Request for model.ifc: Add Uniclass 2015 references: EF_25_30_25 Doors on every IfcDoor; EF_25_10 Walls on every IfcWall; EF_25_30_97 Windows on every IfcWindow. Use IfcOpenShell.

First a look at what the model holds.

```python
import ifcopenshell

model = ifcopenshell.open("model.ifc")
print(model.schema)
print("classifications:", [c.Name for c in model.by_type("IfcClassification")])
for ifc_class in ("IfcDoor", "IfcRoof", "IfcStair", "IfcWall", "IfcWindow"):
    print(ifc_class, len(model.by_type(ifc_class)))
```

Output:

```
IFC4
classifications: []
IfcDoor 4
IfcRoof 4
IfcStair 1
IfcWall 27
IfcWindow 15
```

```python
import ifcopenshell
import ifcopenshell.api.classification

model = ifcopenshell.open("model.ifc")

system = ifcopenshell.api.classification.add_classification(model, classification="Uniclass 2015")

codes = {
    "IfcDoor": ("EF_25_30_25", "Doors"),
    "IfcWall": ("EF_25_10", "Walls"),
    "IfcWindow": ("EF_25_30_97", "Windows"),
}
for ifc_class, (code, name) in codes.items():
    products = model.by_type(ifc_class)
    ifcopenshell.api.classification.add_reference(
        model, products=products, classification=system, identification=code, name=name
    )
    print(code, len(products))

model.write("model_edited.ifc")
```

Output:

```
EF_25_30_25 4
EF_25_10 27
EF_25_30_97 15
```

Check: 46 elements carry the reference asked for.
